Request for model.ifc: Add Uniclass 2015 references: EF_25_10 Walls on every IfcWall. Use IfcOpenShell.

First a look at what the model holds.

```python
import ifcopenshell

model = ifcopenshell.open("model.ifc")
print(model.schema)
print("classifications:", [c.Name for c in model.by_type("IfcClassification")])
for ifc_class in ("IfcDoor", "IfcRoof", "IfcStair", "IfcWall", "IfcWindow"):
    print(ifc_class, len(model.by_type(ifc_class)))
```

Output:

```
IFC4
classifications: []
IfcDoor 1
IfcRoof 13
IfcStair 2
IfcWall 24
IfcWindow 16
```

```python
import ifcopenshell
import ifcopenshell.api.classification

model = ifcopenshell.open("model.ifc")

system = ifcopenshell.api.classification.add_classification(model, classification="Uniclass 2015")

codes = {
    "IfcWall": ("EF_25_10", "Walls"),
}
for ifc_class, (code, name) in codes.items():
    products = model.by_type(ifc_class)
    ifcopenshell.api.classification.add_reference(
        model, products=products, classification=system, identification=code, name=name
    )
    print(code, len(products))

model.write("model_updated.ifc")
```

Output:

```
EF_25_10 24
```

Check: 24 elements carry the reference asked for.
